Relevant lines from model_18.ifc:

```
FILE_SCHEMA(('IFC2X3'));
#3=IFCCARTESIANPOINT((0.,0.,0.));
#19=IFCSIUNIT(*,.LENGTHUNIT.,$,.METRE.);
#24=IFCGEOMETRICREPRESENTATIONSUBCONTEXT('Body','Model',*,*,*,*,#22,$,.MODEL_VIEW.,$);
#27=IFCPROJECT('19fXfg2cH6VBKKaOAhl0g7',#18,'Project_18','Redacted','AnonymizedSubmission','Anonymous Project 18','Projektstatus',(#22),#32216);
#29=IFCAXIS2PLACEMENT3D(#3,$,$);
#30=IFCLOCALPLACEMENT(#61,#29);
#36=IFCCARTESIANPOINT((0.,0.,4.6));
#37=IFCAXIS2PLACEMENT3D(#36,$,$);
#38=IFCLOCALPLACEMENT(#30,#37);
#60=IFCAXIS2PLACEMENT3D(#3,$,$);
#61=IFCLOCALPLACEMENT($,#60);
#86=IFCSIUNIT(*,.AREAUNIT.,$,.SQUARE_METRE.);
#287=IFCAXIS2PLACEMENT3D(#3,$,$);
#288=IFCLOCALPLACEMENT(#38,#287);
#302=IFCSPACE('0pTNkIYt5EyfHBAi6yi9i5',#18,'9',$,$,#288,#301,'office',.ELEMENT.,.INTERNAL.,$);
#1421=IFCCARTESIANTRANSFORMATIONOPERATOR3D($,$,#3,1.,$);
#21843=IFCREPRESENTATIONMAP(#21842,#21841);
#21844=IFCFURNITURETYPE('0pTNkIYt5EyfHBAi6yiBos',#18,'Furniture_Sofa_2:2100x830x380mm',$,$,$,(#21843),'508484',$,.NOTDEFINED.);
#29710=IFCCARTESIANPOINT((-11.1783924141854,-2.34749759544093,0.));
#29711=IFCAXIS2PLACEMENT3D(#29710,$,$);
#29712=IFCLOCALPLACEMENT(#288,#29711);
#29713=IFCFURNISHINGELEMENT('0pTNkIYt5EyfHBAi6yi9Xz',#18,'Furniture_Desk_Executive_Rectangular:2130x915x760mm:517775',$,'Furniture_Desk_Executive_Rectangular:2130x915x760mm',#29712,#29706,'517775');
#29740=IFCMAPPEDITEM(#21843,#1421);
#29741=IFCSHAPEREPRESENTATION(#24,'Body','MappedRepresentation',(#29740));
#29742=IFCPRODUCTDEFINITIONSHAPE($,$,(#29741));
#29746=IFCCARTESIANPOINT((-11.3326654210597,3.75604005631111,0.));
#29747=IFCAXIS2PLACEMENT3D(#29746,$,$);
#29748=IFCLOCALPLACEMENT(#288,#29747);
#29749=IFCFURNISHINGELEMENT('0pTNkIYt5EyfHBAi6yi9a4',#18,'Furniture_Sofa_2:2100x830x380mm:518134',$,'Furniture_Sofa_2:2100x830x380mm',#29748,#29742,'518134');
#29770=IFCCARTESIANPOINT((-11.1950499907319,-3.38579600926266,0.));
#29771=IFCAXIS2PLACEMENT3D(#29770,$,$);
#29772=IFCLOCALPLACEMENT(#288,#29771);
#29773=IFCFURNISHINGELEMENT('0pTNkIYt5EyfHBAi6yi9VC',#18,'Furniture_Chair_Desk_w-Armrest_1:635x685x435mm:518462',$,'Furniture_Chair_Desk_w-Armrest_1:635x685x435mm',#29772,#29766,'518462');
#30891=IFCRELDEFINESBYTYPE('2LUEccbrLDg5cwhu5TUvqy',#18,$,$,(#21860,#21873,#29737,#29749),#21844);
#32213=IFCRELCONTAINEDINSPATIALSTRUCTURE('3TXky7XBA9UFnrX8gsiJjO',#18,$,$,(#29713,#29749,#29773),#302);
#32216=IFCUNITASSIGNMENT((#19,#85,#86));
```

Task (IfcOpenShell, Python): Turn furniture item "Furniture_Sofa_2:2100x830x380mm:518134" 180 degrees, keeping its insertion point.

```python
import ifcopenshell
import ifcopenshell.api.geometry
import ifcopenshell.util.placement

model = ifcopenshell.open("model_18.ifc")

item = model.by_guid("0pTNkIYt5EyfHBAi6yi9a4")
matrix = ifcopenshell.util.placement.get_local_placement(item.ObjectPlacement)
matrix = matrix @ ifcopenshell.util.placement.rotation(180, "Z")
ifcopenshell.api.geometry.edit_object_placement(model, product=item, matrix=matrix, is_si=False)

print(ifcopenshell.util.placement.get_local_placement(item.ObjectPlacement).round(3) + 0.0)

model.write("model_18_v2.ifc")
```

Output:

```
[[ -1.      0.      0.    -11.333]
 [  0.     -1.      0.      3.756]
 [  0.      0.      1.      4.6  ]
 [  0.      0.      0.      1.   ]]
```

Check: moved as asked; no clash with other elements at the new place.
